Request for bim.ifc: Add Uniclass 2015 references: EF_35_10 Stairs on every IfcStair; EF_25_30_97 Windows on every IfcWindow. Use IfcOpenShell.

First a look at what the model holds.

```python
import ifcopenshell

model = ifcopenshell.open("bim.ifc")
print(model.schema)
print("classifications:", [c.Name for c in model.by_type("IfcClassification")])
for ifc_class in ("IfcDoor", "IfcRoof", "IfcStair", "IfcWall", "IfcWindow"):
    print(ifc_class, len(model.by_type(ifc_class)))
```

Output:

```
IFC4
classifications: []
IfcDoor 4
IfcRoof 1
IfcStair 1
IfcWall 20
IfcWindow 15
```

```python
import ifcopenshell
import ifcopenshell.api.classification

model = ifcopenshell.open("bim.ifc")

system = ifcopenshell.api.classification.add_classification(model, classification="Uniclass 2015")

codes = {
    "IfcStair": ("EF_35_10", "Stairs"),
    "IfcWindow": ("EF_25_30_97", "Windows"),
}
for ifc_class, (code, name) in codes.items():
    products = model.by_type(ifc_class)
    ifcopenshell.api.classification.add_reference(
        model, products=products, classification=system, identification=code, name=name
    )
    print(code, len(products))

model.write("bim_updated.ifc")
```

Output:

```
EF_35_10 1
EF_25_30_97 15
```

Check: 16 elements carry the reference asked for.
